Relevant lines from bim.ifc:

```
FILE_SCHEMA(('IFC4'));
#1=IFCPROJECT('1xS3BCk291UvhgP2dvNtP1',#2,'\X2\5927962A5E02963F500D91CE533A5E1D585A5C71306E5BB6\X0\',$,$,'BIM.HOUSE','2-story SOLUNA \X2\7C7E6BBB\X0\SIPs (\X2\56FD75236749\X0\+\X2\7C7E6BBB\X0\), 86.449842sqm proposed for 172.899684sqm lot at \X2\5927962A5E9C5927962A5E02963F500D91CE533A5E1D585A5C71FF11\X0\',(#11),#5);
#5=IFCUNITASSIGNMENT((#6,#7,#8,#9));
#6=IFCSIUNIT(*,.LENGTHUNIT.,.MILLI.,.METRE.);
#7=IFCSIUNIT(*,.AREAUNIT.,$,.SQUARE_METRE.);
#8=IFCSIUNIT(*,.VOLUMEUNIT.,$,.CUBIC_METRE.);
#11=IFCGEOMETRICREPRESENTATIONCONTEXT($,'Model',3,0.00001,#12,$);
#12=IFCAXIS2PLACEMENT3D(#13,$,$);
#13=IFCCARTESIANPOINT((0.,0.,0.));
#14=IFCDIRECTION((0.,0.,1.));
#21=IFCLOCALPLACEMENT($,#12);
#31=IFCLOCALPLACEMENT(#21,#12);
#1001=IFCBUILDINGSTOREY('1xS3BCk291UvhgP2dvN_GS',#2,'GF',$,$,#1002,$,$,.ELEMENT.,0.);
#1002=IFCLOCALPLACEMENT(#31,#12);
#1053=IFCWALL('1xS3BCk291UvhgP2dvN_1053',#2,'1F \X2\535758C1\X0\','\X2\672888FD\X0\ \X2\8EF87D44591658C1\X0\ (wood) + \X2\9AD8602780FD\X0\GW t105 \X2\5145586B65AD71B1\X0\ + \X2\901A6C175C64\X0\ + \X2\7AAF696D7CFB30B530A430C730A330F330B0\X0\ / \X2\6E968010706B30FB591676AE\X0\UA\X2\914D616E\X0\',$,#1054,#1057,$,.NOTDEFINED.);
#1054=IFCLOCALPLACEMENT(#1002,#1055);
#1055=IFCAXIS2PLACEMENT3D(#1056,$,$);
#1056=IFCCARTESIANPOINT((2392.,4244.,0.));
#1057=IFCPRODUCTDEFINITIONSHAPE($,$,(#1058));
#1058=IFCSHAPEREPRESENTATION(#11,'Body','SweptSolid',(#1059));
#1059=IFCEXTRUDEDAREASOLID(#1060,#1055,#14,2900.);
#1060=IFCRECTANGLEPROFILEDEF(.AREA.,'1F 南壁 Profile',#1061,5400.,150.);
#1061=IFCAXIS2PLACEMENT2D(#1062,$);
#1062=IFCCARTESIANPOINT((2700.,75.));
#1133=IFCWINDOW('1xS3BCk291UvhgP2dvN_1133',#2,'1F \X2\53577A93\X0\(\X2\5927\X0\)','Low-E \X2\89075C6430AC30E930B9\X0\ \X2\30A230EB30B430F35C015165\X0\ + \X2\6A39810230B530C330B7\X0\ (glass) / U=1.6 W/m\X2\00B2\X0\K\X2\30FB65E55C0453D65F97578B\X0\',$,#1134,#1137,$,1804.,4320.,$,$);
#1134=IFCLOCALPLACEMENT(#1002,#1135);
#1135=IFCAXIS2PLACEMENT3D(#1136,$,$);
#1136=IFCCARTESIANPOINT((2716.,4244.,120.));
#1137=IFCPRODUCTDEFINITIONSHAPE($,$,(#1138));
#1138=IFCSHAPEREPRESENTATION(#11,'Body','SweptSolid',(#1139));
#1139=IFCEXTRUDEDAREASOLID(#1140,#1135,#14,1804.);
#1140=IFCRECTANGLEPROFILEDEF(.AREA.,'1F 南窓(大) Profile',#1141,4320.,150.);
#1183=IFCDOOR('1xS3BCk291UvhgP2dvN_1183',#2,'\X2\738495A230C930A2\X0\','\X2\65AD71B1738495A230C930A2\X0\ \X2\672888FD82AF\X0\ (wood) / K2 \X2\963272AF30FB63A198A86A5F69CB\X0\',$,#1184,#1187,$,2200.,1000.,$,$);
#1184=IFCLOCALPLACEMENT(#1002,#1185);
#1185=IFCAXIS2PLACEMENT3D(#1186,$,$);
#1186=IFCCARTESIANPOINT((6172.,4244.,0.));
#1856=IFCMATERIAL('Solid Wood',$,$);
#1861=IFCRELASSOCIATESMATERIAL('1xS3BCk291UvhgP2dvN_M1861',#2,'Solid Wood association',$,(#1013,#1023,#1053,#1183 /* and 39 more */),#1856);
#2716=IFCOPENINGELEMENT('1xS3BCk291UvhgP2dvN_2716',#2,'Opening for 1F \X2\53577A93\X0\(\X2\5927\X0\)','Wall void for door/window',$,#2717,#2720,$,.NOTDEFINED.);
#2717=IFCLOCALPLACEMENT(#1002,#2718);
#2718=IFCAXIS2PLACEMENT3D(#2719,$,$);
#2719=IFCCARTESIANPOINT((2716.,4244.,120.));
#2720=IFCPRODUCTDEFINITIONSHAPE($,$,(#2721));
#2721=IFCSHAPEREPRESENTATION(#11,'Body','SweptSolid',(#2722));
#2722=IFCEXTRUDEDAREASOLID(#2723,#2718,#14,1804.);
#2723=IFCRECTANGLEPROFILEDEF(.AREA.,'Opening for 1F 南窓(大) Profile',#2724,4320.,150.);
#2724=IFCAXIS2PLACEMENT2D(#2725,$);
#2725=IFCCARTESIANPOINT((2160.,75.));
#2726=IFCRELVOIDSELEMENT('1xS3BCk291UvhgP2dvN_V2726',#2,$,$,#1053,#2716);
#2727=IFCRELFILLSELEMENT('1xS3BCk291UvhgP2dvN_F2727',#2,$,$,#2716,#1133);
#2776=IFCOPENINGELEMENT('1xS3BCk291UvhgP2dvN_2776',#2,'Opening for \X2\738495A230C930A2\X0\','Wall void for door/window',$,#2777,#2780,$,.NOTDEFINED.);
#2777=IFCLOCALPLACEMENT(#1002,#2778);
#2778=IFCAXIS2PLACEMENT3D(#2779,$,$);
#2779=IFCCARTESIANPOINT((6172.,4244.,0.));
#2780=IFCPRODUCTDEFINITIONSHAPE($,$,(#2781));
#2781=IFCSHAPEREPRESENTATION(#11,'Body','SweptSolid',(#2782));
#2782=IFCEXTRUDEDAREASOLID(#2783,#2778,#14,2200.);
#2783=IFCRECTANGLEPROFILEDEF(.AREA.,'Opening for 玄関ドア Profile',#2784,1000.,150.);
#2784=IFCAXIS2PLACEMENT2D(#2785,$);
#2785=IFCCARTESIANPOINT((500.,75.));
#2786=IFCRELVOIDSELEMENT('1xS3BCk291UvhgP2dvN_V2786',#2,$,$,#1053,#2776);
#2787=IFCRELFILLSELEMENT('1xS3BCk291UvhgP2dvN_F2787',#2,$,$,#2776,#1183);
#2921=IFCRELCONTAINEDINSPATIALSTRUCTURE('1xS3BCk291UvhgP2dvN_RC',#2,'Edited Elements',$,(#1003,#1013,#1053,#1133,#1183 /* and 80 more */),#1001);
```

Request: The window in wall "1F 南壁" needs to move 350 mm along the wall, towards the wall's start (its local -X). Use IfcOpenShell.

```python
import ifcopenshell
import ifcopenshell.api.geometry
import ifcopenshell.util.placement
import ifcopenshell.util.unit

model = ifcopenshell.open("bim.ifc")
unit_scale = ifcopenshell.util.unit.calculate_unit_scale(model)

window = model.by_guid("1xS3BCk291UvhgP2dvN_1133")
opening = window.FillsVoids[0].RelatingOpeningElement
wall = opening.VoidsElements[0].RelatingBuildingElement

wall_matrix = ifcopenshell.util.placement.get_local_placement(wall.ObjectPlacement)
shift = wall_matrix[:3, 0] * -0.35 / unit_scale
before = ifcopenshell.util.placement.get_local_placement(window.ObjectPlacement)[:3, 3].copy()

# The window is not placed relative to its opening, so move both.
for product in (opening, window):
    matrix = ifcopenshell.util.placement.get_local_placement(product.ObjectPlacement)
    matrix[:3, 3] += shift
    ifcopenshell.api.geometry.edit_object_placement(model, product=product, matrix=matrix, is_si=False)

after = ifcopenshell.util.placement.get_local_placement(window.ObjectPlacement)[:3, 3]
print("window moved by", (after - before).round(3) + 0.0)

model.write("bim-out.ifc")
```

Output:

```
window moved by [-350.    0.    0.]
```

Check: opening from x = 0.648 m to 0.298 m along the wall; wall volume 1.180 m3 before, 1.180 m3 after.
